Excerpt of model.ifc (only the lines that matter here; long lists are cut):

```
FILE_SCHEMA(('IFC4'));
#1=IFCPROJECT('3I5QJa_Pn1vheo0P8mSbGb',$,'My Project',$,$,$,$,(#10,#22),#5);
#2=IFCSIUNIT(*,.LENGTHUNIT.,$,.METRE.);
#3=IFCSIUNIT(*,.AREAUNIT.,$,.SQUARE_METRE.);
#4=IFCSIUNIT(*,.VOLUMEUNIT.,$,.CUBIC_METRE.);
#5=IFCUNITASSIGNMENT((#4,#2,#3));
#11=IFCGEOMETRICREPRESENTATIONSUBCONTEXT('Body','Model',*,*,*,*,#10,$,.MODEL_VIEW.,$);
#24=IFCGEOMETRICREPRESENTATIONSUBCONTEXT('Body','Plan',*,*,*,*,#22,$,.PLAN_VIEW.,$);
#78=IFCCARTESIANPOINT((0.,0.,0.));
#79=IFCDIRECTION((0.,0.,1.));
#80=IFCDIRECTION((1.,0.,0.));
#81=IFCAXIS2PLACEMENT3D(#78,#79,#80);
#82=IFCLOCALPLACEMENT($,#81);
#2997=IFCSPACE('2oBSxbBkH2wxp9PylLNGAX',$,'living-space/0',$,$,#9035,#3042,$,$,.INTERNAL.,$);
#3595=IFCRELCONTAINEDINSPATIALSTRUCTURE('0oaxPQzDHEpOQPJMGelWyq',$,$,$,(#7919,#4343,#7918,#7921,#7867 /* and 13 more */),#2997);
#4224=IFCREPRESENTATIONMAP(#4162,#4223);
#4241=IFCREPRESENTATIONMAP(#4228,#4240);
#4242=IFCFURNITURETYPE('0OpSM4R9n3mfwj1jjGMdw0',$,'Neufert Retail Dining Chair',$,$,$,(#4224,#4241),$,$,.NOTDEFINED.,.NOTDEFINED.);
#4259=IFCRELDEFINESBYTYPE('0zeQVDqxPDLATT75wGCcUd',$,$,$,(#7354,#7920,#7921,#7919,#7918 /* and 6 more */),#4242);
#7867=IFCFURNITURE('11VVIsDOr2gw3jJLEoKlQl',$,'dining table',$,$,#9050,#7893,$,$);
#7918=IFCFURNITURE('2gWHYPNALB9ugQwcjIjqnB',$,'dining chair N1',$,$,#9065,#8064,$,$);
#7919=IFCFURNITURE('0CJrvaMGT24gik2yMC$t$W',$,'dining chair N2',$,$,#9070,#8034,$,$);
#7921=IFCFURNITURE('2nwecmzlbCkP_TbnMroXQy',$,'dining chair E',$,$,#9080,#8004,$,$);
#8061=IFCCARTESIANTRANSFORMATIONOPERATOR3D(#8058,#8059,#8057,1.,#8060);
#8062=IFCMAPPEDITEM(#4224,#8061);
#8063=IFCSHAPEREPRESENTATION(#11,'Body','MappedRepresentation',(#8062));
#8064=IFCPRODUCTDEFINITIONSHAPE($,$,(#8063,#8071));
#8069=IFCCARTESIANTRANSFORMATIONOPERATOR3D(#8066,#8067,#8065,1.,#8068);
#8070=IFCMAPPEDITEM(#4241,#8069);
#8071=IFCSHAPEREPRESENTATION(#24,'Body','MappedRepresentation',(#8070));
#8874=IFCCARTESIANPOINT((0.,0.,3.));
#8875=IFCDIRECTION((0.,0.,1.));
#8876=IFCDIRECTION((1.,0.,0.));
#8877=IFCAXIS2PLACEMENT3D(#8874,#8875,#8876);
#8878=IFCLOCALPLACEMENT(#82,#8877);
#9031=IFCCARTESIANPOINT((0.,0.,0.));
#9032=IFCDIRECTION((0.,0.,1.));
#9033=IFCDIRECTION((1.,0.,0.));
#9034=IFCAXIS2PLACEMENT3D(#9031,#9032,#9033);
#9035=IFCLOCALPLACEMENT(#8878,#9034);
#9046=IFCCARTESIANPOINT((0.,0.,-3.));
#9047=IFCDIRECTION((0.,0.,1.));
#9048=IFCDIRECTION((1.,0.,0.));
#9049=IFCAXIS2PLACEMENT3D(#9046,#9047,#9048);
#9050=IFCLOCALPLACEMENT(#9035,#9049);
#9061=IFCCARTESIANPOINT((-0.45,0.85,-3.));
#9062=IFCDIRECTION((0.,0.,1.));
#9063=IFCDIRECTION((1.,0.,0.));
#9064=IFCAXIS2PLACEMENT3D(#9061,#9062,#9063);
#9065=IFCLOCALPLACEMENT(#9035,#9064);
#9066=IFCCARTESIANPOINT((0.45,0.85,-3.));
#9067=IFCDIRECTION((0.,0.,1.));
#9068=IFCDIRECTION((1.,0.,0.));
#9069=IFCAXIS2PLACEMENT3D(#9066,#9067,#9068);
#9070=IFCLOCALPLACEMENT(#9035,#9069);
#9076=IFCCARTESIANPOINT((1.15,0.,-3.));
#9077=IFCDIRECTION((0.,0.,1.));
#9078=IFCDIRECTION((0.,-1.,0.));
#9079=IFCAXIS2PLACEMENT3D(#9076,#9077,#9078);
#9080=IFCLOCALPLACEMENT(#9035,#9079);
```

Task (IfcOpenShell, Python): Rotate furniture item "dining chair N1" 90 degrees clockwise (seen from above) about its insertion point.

```python
import ifcopenshell
import ifcopenshell.api.geometry
import ifcopenshell.util.placement

model = ifcopenshell.open("model.ifc")

item = model.by_guid("2gWHYPNALB9ugQwcjIjqnB")
matrix = ifcopenshell.util.placement.get_local_placement(item.ObjectPlacement)
matrix = matrix @ ifcopenshell.util.placement.rotation(-90, "Z")
ifcopenshell.api.geometry.edit_object_placement(model, product=item, matrix=matrix, is_si=False)

print(ifcopenshell.util.placement.get_local_placement(item.ObjectPlacement).round(3) + 0.0)

model.write("model_v2.ifc")
```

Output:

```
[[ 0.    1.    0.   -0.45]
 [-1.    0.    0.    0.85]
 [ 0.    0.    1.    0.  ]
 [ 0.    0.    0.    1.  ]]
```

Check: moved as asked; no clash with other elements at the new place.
